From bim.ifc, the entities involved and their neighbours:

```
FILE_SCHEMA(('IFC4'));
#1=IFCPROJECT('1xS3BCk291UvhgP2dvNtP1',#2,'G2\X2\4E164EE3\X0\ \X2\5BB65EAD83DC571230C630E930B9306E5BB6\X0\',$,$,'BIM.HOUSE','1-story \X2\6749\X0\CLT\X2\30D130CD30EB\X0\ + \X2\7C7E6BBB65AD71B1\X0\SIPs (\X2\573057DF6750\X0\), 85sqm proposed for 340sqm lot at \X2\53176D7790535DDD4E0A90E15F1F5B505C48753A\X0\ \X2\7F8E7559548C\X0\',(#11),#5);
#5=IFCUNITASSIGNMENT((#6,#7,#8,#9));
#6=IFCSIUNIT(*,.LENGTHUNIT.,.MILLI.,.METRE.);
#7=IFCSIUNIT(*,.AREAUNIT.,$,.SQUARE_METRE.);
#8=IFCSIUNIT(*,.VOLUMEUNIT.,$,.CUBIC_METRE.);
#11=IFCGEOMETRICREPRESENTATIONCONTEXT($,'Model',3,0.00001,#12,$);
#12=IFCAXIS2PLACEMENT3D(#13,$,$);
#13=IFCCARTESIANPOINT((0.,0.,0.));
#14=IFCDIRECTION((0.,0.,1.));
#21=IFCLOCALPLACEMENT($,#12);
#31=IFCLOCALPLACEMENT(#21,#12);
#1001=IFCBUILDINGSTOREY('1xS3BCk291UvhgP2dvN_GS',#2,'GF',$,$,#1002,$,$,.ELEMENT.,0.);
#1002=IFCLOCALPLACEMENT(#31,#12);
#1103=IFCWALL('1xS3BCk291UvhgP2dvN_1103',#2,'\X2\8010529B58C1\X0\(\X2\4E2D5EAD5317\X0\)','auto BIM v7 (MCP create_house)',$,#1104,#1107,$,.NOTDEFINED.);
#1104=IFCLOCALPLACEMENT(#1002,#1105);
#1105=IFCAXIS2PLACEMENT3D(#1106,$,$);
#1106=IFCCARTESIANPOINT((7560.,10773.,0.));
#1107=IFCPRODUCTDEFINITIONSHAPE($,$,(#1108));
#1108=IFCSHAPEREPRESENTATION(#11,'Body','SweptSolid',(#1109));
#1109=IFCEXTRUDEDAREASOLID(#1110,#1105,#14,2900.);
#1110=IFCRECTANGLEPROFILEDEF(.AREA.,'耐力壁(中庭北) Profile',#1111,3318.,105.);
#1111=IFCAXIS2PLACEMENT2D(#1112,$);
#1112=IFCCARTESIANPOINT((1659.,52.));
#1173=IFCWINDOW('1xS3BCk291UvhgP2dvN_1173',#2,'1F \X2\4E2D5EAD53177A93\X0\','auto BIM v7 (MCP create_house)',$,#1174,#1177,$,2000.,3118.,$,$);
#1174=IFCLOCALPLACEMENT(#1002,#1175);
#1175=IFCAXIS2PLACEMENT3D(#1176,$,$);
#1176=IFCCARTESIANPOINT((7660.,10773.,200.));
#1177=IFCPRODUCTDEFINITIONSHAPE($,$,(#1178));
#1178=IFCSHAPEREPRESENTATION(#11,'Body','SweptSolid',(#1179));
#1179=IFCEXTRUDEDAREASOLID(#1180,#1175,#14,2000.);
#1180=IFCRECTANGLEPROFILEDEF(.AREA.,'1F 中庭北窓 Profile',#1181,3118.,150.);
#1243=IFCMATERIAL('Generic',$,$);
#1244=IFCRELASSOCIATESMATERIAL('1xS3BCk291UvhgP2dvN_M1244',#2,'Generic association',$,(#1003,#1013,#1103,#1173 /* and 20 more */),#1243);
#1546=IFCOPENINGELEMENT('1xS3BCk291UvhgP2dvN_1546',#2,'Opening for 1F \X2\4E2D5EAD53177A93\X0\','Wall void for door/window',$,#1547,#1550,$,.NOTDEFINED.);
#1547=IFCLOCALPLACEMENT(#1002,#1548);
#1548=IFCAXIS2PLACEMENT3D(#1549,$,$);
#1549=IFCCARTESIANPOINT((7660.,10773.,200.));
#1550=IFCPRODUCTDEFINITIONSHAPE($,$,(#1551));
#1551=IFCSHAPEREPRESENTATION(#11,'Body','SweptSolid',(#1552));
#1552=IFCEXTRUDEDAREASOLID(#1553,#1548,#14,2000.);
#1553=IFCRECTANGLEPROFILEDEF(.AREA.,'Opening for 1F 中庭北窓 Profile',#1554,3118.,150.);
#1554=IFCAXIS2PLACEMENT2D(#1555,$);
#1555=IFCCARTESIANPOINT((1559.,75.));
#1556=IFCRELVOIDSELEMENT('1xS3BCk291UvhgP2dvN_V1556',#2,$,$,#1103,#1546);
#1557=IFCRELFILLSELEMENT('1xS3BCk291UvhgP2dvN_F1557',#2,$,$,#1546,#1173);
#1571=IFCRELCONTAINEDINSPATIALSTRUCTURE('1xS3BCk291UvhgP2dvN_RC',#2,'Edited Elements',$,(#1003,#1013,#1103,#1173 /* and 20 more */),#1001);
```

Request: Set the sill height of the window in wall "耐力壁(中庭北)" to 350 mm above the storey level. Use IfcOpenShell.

```python
import numpy as np
import ifcopenshell
import ifcopenshell.api.geometry
import ifcopenshell.geom
import ifcopenshell.util.element
import ifcopenshell.util.placement
import ifcopenshell.util.shape
import ifcopenshell.util.unit

model = ifcopenshell.open("bim.ifc")
unit_scale = ifcopenshell.util.unit.calculate_unit_scale(model)

window = model.by_guid("1xS3BCk291UvhgP2dvN_1173")
opening = window.FillsVoids[0].RelatingOpeningElement
storey = ifcopenshell.util.element.get_container(window, ifc_class="IfcBuildingStorey")
level = ifcopenshell.util.placement.get_local_placement(storey.ObjectPlacement)[2, 3]

# The opening's origin need not be at the sill, so measure its lowest point.
shape = ifcopenshell.geom.create_shape(ifcopenshell.geom.settings(), opening)
bottom = ifcopenshell.util.shape.get_shape_bottom_elevation(shape, shape.geometry) / unit_scale
dz = level + 0.35 / unit_scale - bottom

shift = np.array([0.0, 0.0, dz])
# The window is not placed relative to its opening, so move both.
for product in (opening, window):
    matrix = ifcopenshell.util.placement.get_local_placement(product.ObjectPlacement)
    matrix[:3, 3] += shift
    ifcopenshell.api.geometry.edit_object_placement(model, product=product, matrix=matrix, is_si=False)

print(f"moved by {dz * unit_scale:+.3f} m")

model.write("bim_rev.ifc")
```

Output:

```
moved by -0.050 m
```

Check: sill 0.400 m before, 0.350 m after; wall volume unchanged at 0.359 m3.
